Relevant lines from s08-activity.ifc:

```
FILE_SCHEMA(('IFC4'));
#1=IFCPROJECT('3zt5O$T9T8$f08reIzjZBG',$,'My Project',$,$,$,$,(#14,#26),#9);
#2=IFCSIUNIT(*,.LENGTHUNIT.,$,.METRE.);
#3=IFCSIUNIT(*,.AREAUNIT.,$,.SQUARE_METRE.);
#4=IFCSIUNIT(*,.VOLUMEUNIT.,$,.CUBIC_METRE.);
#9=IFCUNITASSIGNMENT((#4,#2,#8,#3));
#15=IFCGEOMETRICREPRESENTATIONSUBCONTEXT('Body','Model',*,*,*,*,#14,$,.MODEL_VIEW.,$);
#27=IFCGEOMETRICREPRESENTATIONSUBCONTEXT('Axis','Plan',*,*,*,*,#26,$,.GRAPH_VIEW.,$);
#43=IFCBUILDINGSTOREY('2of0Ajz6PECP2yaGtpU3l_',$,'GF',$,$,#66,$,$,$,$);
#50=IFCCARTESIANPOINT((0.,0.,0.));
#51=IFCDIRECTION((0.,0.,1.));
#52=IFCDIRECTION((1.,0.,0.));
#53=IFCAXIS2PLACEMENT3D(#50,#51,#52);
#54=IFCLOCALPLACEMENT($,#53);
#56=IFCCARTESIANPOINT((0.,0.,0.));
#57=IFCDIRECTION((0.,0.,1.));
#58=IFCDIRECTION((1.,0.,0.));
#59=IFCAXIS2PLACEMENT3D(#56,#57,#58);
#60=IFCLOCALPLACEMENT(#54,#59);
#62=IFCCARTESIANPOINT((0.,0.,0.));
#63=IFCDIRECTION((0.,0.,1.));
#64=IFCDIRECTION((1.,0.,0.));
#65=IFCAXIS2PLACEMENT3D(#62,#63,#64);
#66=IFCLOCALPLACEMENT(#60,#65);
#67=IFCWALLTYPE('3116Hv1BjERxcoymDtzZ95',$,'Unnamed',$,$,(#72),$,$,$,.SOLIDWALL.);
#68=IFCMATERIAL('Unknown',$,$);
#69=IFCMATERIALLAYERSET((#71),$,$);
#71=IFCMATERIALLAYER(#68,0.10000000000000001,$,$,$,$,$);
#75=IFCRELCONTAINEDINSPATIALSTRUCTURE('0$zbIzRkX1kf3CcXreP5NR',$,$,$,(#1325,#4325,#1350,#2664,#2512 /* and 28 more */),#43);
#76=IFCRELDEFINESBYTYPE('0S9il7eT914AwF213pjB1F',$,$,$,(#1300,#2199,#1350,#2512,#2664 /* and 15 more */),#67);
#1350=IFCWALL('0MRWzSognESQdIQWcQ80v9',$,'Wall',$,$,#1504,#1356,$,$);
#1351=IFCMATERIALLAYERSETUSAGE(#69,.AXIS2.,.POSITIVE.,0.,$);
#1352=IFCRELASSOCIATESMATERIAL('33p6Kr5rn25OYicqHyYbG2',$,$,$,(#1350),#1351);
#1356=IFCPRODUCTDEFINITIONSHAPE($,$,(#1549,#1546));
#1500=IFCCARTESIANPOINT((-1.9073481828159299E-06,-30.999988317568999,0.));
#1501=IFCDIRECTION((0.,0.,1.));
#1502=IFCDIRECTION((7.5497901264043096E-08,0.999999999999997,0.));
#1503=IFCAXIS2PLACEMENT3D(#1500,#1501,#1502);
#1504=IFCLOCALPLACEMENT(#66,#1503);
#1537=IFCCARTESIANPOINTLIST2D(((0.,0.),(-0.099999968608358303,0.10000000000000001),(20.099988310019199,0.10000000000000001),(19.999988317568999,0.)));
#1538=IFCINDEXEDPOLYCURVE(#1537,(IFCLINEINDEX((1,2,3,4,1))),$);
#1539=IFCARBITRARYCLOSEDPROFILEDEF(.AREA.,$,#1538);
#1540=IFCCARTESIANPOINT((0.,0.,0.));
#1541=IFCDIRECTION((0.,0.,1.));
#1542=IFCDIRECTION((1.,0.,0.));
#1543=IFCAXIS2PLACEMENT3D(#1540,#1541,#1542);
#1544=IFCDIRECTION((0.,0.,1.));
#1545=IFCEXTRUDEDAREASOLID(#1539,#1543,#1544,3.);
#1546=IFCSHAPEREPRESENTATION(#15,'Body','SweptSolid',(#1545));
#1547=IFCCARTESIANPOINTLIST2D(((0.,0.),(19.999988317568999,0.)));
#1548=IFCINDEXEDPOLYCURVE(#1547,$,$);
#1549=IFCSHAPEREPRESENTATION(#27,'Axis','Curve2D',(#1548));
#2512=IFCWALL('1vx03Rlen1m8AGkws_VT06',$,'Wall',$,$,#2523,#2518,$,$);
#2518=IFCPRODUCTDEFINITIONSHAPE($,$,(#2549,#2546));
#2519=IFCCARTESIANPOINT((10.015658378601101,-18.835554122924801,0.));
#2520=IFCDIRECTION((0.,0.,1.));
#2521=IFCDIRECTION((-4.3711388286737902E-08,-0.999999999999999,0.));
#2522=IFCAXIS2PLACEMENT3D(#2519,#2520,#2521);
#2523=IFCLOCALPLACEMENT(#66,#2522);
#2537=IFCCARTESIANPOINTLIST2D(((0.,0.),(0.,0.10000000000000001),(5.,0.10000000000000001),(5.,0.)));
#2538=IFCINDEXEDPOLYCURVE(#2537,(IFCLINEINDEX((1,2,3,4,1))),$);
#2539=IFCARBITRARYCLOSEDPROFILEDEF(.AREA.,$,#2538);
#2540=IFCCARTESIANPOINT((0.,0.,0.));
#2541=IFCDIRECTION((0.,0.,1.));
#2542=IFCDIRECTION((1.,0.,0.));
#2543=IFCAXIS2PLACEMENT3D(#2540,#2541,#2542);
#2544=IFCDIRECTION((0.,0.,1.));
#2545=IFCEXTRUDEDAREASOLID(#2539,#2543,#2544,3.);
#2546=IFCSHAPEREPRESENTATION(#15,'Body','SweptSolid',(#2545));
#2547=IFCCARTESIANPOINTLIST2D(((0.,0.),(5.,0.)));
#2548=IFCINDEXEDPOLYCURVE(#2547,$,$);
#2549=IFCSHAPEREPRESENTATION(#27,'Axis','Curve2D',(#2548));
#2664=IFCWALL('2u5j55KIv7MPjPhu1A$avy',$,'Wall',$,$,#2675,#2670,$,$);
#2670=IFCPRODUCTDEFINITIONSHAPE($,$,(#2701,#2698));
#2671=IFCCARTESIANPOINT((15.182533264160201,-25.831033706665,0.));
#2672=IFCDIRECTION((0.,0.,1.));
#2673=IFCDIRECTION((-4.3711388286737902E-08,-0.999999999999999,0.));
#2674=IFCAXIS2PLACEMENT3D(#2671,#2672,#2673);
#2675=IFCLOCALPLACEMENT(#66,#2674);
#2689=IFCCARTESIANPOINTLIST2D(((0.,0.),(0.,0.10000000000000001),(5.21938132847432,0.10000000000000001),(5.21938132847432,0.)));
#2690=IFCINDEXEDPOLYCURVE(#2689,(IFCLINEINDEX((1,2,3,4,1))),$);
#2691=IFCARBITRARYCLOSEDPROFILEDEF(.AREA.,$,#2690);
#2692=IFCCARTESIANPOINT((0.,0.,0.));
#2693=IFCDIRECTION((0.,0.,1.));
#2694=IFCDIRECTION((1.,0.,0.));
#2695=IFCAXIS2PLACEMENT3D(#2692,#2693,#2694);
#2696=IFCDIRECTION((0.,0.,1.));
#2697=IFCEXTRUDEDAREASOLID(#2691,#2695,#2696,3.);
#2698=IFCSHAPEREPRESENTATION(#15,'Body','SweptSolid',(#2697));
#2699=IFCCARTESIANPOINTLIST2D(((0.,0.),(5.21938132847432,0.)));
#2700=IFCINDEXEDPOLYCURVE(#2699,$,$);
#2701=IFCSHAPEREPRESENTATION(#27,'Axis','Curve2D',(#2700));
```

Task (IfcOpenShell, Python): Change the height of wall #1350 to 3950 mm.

```python
import ifcopenshell
import ifcopenshell.geom
import ifcopenshell.util.representation
import ifcopenshell.util.shape

model = ifcopenshell.open("s08-activity.ifc")
settings = ifcopenshell.geom.settings()


def volume(element):
    """Net volume in cubic metres, openings subtracted."""
    shape = ifcopenshell.geom.create_shape(settings, element)
    return ifcopenshell.util.shape.get_volume(shape.geometry)


wall = model.by_id(1350)
before = volume(wall)

body = ifcopenshell.util.representation.get_representation(wall, "Model", "Body")
solid = body.Items[0]
old_height = solid.Depth
solid.Depth = 3.95
after = volume(wall)

print(f"height {old_height:g} -> {solid.Depth:g}, volume {before:.3f} -> {after:.3f} m3")

model.write("s08-activity_updated.ifc")
```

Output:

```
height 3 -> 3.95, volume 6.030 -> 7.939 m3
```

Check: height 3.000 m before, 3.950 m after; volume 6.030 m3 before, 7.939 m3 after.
